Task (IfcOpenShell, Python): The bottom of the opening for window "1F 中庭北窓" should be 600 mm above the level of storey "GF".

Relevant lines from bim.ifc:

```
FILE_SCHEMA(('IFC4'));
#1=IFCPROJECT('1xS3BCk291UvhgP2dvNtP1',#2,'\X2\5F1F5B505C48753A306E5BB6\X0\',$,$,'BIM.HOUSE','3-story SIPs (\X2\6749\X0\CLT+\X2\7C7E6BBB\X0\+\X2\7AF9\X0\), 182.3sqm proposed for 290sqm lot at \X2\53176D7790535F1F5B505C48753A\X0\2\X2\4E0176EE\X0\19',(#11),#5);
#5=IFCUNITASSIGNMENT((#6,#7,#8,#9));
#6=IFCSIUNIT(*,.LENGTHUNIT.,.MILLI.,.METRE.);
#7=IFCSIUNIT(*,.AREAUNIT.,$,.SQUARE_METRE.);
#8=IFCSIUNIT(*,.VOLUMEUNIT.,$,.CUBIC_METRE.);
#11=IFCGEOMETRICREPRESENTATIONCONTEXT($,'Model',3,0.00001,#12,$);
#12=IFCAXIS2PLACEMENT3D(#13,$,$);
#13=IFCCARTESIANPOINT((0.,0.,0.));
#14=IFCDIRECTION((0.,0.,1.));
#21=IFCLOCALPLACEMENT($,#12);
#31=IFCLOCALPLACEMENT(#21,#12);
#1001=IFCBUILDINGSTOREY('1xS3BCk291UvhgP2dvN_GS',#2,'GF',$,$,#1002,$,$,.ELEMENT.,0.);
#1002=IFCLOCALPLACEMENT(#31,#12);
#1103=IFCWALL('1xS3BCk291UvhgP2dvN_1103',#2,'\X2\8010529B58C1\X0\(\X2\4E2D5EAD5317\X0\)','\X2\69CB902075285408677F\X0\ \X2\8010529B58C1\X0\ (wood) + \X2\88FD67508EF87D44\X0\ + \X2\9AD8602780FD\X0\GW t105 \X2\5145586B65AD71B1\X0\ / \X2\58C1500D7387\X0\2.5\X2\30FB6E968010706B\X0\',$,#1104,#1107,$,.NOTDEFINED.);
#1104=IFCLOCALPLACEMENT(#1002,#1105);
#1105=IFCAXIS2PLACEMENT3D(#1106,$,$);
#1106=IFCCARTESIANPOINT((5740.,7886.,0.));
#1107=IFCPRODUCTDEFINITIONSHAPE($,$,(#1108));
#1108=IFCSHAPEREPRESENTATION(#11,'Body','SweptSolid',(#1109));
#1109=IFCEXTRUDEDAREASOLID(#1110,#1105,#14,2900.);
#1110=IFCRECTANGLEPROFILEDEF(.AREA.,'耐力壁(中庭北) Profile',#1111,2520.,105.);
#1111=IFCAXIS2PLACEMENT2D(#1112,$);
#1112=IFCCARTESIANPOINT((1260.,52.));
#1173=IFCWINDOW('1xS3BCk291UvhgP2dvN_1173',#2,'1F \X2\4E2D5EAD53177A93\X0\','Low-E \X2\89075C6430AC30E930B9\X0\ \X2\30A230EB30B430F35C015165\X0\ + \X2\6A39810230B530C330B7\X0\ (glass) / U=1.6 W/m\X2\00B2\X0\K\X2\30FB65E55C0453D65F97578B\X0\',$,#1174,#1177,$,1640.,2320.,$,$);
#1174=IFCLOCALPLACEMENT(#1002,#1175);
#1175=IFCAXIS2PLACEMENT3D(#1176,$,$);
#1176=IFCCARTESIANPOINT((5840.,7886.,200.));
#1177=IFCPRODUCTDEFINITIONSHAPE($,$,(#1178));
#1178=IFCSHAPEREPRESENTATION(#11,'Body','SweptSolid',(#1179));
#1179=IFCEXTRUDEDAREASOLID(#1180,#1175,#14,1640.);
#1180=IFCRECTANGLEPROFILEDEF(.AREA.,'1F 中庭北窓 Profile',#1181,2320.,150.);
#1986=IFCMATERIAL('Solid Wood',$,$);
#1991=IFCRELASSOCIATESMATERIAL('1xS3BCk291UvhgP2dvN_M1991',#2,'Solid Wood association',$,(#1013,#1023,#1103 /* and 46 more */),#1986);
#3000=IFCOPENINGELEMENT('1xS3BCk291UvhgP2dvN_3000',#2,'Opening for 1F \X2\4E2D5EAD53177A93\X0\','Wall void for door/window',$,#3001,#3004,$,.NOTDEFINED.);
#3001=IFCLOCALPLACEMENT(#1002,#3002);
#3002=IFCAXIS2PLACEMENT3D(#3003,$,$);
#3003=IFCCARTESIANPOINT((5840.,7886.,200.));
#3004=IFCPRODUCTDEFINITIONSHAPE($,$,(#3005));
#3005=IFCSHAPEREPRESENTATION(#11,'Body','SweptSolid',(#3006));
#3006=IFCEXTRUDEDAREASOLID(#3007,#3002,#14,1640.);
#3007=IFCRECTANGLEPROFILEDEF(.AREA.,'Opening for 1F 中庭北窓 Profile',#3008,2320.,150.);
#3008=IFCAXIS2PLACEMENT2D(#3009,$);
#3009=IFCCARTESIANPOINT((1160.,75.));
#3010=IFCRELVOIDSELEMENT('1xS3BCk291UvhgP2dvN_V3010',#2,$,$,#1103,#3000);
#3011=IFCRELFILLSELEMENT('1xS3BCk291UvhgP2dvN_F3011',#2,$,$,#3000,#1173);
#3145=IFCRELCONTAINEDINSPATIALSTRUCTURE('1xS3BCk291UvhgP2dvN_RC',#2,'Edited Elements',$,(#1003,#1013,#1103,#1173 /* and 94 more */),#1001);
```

```python
import numpy as np
import ifcopenshell
import ifcopenshell.api.geometry
import ifcopenshell.geom
import ifcopenshell.util.element
import ifcopenshell.util.placement
import ifcopenshell.util.shape
import ifcopenshell.util.unit

model = ifcopenshell.open("bim.ifc")
unit_scale = ifcopenshell.util.unit.calculate_unit_scale(model)

window = model.by_guid("1xS3BCk291UvhgP2dvN_1173")
opening = window.FillsVoids[0].RelatingOpeningElement
storey = ifcopenshell.util.element.get_container(window, ifc_class="IfcBuildingStorey")
level = ifcopenshell.util.placement.get_local_placement(storey.ObjectPlacement)[2, 3]

# The opening's origin need not be at the sill, so measure its lowest point.
shape = ifcopenshell.geom.create_shape(ifcopenshell.geom.settings(), opening)
bottom = ifcopenshell.util.shape.get_shape_bottom_elevation(shape, shape.geometry) / unit_scale
dz = level + 600.0 - bottom

shift = np.array([0.0, 0.0, dz])
# The window is not placed relative to its opening, so move both.
for product in (opening, window):
    matrix = ifcopenshell.util.placement.get_local_placement(product.ObjectPlacement)
    matrix[:3, 3] += shift
    ifcopenshell.api.geometry.edit_object_placement(model, product=product, matrix=matrix, is_si=False)

print(f"moved by {dz * unit_scale:+.3f} m")

model.write("bim_rev.ifc")
```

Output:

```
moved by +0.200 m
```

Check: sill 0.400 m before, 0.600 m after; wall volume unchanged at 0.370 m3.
